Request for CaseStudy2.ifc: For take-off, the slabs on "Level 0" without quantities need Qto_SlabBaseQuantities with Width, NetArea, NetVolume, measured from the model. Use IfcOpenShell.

First a look at what the model holds.

```python
import ifcopenshell
import ifcopenshell.util.element
import ifcopenshell.util.unit

model = ifcopenshell.open("CaseStudy2.ifc")
print(model.schema)
for unit_type in ("LENGTHUNIT", "AREAUNIT", "VOLUMEUNIT"):
    print(unit_type, ifcopenshell.util.unit.calculate_unit_scale(model, unit_type))
storey = next(s for s in model.by_type("IfcBuildingStorey") if s.Name == "Level 0")
slabs = [e for e in ifcopenshell.util.element.get_decomposition(storey) if e.is_a("IfcSlab")]
for e in sorted(slabs, key=lambda e: e.id()):
    print(e.id(), e.is_a(), e.Name, list(ifcopenshell.util.element.get_psets(e, qtos_only=True)), sep=" | ")
```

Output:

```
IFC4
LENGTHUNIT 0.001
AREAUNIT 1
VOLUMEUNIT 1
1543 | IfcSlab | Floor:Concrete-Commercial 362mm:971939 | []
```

```python
import ifcopenshell
import ifcopenshell.api.pset
import ifcopenshell.geom
import ifcopenshell.util.element
import ifcopenshell.util.shape
import ifcopenshell.util.unit

model = ifcopenshell.open("CaseStudy2.ifc")
unit_scale = ifcopenshell.util.unit.calculate_unit_scale(model)
area_scale = ifcopenshell.util.unit.calculate_unit_scale(model, "AREAUNIT")
volume_scale = ifcopenshell.util.unit.calculate_unit_scale(model, "VOLUMEUNIT")
settings = ifcopenshell.geom.settings()

storey = next(s for s in model.by_type("IfcBuildingStorey") if s.Name == "Level 0")
slabs = [e for e in ifcopenshell.util.element.get_decomposition(storey) if e.is_a("IfcSlab")]

for e in sorted(slabs, key=lambda e: e.id()):
    if ifcopenshell.util.element.get_psets(e, qtos_only=True, should_inherit=False):
        continue
    # Geometry comes back in metres, in the element's own axes.
    shape = ifcopenshell.geom.create_shape(settings, e)
    values = {
        "Width": ifcopenshell.util.shape.get_z(shape.geometry) / unit_scale,
        "NetArea": ifcopenshell.util.shape.get_footprint_area(shape.geometry) / area_scale,
        "NetVolume": ifcopenshell.util.shape.get_volume(shape.geometry) / volume_scale,
    }
    qto = ifcopenshell.api.pset.add_qto(model, product=e, name="Qto_SlabBaseQuantities")
    ifcopenshell.api.pset.edit_qto(model, qto=qto, properties=values)
    print(e.id(), {k: round(v, 3) for k, v in values.items()})

model.write("CaseStudy2_edited.ifc")
```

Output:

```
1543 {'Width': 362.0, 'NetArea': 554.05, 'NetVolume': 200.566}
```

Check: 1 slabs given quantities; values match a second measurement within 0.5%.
